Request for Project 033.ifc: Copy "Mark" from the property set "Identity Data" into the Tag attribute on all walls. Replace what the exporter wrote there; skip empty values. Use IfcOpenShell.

First a look at what the model holds.

```python
import ifcopenshell
import ifcopenshell.util.element

model = ifcopenshell.open("Project 033.ifc")
print(model.schema)
walls = model.by_type("IfcWall")
print(len(walls), "walls")
for e in walls[:8]:
    source = ifcopenshell.util.element.get_pset(e, "Identity Data", "Mark")
    target = e.Tag
    print(e.id(), repr(source), repr(target), sep=" | ")
```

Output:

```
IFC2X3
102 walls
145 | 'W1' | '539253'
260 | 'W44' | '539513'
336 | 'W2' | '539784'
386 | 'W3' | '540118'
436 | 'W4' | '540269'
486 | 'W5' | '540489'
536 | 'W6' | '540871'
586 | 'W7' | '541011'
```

```python
import ifcopenshell
import ifcopenshell.util.element

model = ifcopenshell.open("Project 033.ifc")

count = 0
for e in model.by_type("IfcWall"):
    value = ifcopenshell.util.element.get_pset(e, "Identity Data", "Mark")
    current = e.Tag
    if not value or not value.strip() or current == value:
        continue
    e.Tag = value
    count += 1

print(count, "walls updated")

model.write("Project 033_v2.ifc")
```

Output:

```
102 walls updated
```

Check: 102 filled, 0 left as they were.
